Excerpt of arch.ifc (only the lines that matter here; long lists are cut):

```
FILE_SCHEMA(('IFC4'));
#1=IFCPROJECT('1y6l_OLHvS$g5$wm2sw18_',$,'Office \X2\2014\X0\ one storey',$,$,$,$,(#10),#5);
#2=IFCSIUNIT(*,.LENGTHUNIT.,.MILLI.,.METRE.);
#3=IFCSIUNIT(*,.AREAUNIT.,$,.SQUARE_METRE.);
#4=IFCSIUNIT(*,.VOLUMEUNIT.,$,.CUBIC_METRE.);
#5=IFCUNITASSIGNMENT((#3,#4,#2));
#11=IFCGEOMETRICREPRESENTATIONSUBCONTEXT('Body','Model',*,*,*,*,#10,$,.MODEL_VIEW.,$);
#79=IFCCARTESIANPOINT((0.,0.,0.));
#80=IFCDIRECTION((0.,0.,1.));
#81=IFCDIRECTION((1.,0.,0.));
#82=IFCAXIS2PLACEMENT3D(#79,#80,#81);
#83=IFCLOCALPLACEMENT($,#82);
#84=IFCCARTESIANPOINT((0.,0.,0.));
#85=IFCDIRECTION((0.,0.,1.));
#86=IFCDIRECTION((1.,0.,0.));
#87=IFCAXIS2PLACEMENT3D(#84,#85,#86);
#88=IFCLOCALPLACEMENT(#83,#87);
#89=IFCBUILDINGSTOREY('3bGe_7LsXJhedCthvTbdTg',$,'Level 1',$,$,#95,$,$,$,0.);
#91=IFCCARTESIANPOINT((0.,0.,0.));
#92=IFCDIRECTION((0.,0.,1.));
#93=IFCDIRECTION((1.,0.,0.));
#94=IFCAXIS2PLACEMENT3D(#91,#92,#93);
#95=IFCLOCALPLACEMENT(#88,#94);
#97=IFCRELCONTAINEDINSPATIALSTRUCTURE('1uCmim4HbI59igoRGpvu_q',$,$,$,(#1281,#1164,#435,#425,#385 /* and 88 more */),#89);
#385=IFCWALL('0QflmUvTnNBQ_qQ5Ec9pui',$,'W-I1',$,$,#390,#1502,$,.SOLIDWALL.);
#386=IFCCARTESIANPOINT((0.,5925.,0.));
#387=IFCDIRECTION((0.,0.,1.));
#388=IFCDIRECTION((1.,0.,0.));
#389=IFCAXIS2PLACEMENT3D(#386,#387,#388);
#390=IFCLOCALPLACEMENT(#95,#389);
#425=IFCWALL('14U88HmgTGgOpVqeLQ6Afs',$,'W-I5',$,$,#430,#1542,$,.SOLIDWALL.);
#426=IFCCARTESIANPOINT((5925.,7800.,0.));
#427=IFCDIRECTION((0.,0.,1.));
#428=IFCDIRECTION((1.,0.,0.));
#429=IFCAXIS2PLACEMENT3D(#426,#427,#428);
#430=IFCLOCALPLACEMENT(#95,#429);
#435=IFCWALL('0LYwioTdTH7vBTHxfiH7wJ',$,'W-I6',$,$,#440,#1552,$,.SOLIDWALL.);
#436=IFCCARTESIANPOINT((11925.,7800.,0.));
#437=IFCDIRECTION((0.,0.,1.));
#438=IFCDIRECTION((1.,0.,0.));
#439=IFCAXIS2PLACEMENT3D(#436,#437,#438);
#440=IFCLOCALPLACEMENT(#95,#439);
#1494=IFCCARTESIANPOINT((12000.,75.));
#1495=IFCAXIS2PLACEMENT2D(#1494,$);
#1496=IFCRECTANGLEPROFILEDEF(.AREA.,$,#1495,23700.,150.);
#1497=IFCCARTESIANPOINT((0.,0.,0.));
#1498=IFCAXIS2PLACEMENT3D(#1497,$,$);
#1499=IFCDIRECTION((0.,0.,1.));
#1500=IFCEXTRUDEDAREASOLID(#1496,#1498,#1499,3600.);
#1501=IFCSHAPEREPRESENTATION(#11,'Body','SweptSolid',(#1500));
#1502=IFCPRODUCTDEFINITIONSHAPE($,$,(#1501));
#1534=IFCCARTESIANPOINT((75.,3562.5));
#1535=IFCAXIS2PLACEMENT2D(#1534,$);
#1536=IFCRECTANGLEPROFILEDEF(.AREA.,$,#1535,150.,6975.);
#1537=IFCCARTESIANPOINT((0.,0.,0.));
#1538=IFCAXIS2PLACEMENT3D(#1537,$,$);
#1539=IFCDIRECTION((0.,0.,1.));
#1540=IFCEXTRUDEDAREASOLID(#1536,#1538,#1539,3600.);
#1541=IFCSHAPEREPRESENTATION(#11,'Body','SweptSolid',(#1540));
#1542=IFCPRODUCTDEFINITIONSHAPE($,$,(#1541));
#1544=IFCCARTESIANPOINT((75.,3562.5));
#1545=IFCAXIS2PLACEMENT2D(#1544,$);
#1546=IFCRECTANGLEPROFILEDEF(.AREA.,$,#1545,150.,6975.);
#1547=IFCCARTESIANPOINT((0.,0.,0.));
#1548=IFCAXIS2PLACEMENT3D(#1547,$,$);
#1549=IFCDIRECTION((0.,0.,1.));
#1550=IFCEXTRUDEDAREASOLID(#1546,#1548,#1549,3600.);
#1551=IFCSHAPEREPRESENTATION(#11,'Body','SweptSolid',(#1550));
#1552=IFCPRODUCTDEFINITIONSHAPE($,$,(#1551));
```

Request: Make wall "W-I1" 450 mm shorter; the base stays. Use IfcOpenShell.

```python
import ifcopenshell
import ifcopenshell.geom
import ifcopenshell.util.representation
import ifcopenshell.util.shape
import ifcopenshell.util.unit

model = ifcopenshell.open("arch.ifc")
unit_scale = ifcopenshell.util.unit.calculate_unit_scale(model)
settings = ifcopenshell.geom.settings()


def volume(element):
    """Net volume in cubic metres, openings subtracted."""
    shape = ifcopenshell.geom.create_shape(settings, element)
    return ifcopenshell.util.shape.get_volume(shape.geometry)


wall = model.by_guid("0QflmUvTnNBQ_qQ5Ec9pui")
before = volume(wall)

body = ifcopenshell.util.representation.get_representation(wall, "Model", "Body")
solid = body.Items[0]
old_height = solid.Depth
solid.Depth -= 0.45 / unit_scale
after = volume(wall)

print(f"height {old_height:g} -> {solid.Depth:g}, volume {before:.3f} -> {after:.3f} m3")

model.write("arch_edited.ifc")
```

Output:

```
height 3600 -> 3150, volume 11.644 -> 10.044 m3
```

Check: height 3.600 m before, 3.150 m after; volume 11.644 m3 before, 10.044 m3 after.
